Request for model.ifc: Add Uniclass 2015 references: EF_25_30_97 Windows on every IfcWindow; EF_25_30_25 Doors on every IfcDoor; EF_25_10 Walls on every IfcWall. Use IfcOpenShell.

First a look at what the model holds.

```python
import ifcopenshell

model = ifcopenshell.open("model.ifc")
print(model.schema)
print("classifications:", [c.Name for c in model.by_type("IfcClassification")])
for ifc_class in ("IfcDoor", "IfcRoof", "IfcStair", "IfcWall", "IfcWindow"):
    print(ifc_class, len(model.by_type(ifc_class)))
```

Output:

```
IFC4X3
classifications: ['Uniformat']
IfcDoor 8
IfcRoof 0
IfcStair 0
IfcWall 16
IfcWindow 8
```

```python
import ifcopenshell
import ifcopenshell.api.classification

model = ifcopenshell.open("model.ifc")

system = ifcopenshell.api.classification.add_classification(model, classification="Uniclass 2015")

codes = {
    "IfcWindow": ("EF_25_30_97", "Windows"),
    "IfcDoor": ("EF_25_30_25", "Doors"),
    "IfcWall": ("EF_25_10", "Walls"),
}
for ifc_class, (code, name) in codes.items():
    products = model.by_type(ifc_class)
    ifcopenshell.api.classification.add_reference(
        model, products=products, classification=system, identification=code, name=name
    )
    print(code, len(products))

model.write("model_edited.ifc")
```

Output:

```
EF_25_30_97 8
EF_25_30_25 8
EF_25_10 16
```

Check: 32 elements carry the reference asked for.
